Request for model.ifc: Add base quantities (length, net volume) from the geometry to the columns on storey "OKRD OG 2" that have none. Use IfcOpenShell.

First a look at what the model holds.

```python
import ifcopenshell
import ifcopenshell.util.element
import ifcopenshell.util.unit

model = ifcopenshell.open("model.ifc")
print(model.schema)
for unit_type in ("LENGTHUNIT", "AREAUNIT", "VOLUMEUNIT"):
    print(unit_type, ifcopenshell.util.unit.calculate_unit_scale(model, unit_type))
storey = next(s for s in model.by_type("IfcBuildingStorey") if s.Name == "OKRD OG 2")
columns = [e for e in ifcopenshell.util.element.get_decomposition(storey) if e.is_a("IfcColumn")]
for e in sorted(columns, key=lambda e: e.id()):
    print(e.id(), e.is_a(), e.Name, list(ifcopenshell.util.element.get_psets(e, qtos_only=True)), sep=" | ")
```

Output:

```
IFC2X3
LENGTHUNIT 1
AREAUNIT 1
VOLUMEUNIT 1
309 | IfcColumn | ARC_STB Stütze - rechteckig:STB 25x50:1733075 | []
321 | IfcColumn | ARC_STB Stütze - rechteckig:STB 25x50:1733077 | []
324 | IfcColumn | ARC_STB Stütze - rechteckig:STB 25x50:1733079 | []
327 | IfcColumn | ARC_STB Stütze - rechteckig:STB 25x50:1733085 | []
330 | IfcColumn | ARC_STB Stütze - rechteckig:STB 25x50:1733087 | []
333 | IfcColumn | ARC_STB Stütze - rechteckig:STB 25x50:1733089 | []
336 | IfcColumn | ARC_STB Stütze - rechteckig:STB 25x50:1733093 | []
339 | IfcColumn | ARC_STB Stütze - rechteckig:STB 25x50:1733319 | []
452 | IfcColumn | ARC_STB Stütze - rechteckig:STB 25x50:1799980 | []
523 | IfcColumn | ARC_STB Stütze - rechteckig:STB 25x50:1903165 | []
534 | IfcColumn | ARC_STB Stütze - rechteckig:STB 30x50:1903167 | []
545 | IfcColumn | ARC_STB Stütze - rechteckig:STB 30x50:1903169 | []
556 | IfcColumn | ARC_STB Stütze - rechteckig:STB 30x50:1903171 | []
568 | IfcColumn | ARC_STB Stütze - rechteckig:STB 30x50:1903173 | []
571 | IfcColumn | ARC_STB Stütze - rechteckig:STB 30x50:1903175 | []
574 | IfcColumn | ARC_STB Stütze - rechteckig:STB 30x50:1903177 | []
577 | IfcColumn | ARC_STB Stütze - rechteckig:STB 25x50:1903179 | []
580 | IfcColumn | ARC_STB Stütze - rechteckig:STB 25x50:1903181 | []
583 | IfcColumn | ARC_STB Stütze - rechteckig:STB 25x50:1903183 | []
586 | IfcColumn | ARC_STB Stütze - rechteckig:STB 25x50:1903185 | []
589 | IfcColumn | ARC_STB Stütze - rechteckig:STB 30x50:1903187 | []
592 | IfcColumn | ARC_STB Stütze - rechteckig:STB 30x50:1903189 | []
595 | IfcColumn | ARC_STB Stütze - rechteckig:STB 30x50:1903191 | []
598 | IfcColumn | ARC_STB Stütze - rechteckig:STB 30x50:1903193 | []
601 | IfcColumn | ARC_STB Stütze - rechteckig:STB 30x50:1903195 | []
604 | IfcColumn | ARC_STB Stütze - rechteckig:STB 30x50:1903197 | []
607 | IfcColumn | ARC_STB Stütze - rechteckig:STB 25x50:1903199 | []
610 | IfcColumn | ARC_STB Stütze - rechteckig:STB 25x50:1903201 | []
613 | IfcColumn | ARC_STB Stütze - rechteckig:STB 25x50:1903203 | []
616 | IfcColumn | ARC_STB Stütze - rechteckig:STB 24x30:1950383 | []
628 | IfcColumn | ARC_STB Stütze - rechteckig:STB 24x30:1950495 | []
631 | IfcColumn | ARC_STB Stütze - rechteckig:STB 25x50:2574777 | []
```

```python
import ifcopenshell
import ifcopenshell.api.pset
import ifcopenshell.geom
import ifcopenshell.util.element
import ifcopenshell.util.shape
import ifcopenshell.util.unit

model = ifcopenshell.open("model.ifc")
unit_scale = ifcopenshell.util.unit.calculate_unit_scale(model)
volume_scale = ifcopenshell.util.unit.calculate_unit_scale(model, "VOLUMEUNIT")
settings = ifcopenshell.geom.settings()

storey = next(s for s in model.by_type("IfcBuildingStorey") if s.Name == "OKRD OG 2")
columns = [e for e in ifcopenshell.util.element.get_decomposition(storey) if e.is_a("IfcColumn")]

for e in sorted(columns, key=lambda e: e.id()):
    if ifcopenshell.util.element.get_psets(e, qtos_only=True, should_inherit=False):
        continue
    # Geometry comes back in metres, in the element's own axes.
    shape = ifcopenshell.geom.create_shape(settings, e)
    values = {
        "Length": ifcopenshell.util.shape.get_z(shape.geometry) / unit_scale,
        "NetVolume": ifcopenshell.util.shape.get_volume(shape.geometry) / volume_scale,
    }
    qto = ifcopenshell.api.pset.add_qto(model, product=e, name="BaseQuantities")
    ifcopenshell.api.pset.edit_qto(model, qto=qto, properties=values)
    print(e.id(), {k: round(v, 3) for k, v in values.items()})

model.write("model-out.ifc")
```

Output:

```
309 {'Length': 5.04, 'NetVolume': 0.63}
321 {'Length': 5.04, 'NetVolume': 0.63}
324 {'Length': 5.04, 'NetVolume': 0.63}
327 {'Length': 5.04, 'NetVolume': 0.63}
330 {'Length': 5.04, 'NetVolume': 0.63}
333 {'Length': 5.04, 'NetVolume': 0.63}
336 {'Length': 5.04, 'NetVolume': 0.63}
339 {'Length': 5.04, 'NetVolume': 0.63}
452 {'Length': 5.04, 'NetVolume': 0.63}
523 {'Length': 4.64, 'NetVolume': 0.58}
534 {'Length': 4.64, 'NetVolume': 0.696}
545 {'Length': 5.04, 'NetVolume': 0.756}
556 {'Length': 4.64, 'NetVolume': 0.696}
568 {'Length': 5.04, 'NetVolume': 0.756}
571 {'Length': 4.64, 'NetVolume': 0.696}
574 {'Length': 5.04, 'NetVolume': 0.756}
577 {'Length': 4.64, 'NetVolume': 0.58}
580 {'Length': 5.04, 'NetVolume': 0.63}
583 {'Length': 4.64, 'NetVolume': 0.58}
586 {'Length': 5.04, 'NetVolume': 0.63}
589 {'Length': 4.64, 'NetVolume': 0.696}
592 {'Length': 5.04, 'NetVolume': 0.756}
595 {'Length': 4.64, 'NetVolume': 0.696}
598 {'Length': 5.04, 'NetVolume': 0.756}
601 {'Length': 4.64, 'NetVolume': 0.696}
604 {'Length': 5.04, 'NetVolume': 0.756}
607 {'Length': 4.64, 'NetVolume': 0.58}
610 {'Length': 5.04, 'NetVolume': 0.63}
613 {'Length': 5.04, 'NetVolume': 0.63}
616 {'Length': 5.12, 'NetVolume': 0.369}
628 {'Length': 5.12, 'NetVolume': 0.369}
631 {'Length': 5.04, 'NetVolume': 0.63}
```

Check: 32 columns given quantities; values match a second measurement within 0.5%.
